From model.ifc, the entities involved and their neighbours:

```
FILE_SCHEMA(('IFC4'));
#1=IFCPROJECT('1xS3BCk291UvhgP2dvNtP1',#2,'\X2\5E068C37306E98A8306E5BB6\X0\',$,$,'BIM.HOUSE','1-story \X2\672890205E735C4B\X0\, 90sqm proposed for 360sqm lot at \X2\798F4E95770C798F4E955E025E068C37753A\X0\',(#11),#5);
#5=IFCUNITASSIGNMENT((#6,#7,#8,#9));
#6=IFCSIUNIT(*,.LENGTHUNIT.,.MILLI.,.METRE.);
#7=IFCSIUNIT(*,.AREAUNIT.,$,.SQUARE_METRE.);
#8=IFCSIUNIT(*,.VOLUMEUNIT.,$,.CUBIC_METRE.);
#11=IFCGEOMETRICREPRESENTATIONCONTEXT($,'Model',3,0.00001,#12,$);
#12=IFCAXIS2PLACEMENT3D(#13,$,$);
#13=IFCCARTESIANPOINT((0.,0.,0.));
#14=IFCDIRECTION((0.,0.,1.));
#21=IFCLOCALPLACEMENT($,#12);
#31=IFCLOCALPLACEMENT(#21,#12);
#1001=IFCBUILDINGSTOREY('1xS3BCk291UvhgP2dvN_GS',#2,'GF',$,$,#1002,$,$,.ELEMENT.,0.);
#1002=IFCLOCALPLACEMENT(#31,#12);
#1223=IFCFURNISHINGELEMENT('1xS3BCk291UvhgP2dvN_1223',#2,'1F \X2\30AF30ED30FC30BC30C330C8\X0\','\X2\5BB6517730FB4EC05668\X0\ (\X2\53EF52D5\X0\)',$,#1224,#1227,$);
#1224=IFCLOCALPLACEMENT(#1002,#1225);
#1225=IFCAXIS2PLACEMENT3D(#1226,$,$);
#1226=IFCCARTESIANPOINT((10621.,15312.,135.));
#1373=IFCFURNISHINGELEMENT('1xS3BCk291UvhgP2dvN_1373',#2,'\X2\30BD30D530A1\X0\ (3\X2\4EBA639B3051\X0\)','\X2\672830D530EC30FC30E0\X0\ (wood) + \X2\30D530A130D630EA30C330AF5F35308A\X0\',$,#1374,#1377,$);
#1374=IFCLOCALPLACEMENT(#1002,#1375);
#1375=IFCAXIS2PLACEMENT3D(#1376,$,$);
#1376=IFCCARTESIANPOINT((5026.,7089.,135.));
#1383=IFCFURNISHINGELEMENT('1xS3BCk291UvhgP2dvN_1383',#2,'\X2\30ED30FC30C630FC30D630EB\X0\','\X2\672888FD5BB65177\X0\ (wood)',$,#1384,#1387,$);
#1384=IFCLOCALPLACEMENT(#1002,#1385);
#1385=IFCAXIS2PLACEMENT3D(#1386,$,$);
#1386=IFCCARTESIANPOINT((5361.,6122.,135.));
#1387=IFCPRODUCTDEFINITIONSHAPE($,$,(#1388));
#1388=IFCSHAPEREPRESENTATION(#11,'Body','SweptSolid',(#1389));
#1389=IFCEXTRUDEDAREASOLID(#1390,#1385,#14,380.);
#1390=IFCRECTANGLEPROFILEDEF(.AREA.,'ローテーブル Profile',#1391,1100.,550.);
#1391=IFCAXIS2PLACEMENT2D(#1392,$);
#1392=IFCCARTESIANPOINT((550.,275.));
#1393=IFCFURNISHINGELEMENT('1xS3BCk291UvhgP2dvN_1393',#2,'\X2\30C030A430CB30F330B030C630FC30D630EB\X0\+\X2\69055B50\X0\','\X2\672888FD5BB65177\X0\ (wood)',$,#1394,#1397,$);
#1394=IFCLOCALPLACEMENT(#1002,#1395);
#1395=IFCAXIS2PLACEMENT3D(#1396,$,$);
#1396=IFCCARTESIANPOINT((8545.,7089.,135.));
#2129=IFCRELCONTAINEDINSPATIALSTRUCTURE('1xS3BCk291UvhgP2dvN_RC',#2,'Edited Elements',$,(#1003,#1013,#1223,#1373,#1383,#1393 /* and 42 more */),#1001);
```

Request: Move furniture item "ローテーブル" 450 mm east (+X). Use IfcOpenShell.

```python
import ifcopenshell
import ifcopenshell.api.geometry
import ifcopenshell.util.placement
import ifcopenshell.util.unit

model = ifcopenshell.open("model.ifc")
unit_scale = ifcopenshell.util.unit.calculate_unit_scale(model)

item = model.by_id(1383)
matrix = ifcopenshell.util.placement.get_local_placement(item.ObjectPlacement)
matrix[0, 3] += 0.45 / unit_scale
ifcopenshell.api.geometry.edit_object_placement(model, product=item, matrix=matrix, is_si=False)

print(ifcopenshell.util.placement.get_local_placement(item.ObjectPlacement).round(3) + 0.0)

model.write("model-out.ifc")
```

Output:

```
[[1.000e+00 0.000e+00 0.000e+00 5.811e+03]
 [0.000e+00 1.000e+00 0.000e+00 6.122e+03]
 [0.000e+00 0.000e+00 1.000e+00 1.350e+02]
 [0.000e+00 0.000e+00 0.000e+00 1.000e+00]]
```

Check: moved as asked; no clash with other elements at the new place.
